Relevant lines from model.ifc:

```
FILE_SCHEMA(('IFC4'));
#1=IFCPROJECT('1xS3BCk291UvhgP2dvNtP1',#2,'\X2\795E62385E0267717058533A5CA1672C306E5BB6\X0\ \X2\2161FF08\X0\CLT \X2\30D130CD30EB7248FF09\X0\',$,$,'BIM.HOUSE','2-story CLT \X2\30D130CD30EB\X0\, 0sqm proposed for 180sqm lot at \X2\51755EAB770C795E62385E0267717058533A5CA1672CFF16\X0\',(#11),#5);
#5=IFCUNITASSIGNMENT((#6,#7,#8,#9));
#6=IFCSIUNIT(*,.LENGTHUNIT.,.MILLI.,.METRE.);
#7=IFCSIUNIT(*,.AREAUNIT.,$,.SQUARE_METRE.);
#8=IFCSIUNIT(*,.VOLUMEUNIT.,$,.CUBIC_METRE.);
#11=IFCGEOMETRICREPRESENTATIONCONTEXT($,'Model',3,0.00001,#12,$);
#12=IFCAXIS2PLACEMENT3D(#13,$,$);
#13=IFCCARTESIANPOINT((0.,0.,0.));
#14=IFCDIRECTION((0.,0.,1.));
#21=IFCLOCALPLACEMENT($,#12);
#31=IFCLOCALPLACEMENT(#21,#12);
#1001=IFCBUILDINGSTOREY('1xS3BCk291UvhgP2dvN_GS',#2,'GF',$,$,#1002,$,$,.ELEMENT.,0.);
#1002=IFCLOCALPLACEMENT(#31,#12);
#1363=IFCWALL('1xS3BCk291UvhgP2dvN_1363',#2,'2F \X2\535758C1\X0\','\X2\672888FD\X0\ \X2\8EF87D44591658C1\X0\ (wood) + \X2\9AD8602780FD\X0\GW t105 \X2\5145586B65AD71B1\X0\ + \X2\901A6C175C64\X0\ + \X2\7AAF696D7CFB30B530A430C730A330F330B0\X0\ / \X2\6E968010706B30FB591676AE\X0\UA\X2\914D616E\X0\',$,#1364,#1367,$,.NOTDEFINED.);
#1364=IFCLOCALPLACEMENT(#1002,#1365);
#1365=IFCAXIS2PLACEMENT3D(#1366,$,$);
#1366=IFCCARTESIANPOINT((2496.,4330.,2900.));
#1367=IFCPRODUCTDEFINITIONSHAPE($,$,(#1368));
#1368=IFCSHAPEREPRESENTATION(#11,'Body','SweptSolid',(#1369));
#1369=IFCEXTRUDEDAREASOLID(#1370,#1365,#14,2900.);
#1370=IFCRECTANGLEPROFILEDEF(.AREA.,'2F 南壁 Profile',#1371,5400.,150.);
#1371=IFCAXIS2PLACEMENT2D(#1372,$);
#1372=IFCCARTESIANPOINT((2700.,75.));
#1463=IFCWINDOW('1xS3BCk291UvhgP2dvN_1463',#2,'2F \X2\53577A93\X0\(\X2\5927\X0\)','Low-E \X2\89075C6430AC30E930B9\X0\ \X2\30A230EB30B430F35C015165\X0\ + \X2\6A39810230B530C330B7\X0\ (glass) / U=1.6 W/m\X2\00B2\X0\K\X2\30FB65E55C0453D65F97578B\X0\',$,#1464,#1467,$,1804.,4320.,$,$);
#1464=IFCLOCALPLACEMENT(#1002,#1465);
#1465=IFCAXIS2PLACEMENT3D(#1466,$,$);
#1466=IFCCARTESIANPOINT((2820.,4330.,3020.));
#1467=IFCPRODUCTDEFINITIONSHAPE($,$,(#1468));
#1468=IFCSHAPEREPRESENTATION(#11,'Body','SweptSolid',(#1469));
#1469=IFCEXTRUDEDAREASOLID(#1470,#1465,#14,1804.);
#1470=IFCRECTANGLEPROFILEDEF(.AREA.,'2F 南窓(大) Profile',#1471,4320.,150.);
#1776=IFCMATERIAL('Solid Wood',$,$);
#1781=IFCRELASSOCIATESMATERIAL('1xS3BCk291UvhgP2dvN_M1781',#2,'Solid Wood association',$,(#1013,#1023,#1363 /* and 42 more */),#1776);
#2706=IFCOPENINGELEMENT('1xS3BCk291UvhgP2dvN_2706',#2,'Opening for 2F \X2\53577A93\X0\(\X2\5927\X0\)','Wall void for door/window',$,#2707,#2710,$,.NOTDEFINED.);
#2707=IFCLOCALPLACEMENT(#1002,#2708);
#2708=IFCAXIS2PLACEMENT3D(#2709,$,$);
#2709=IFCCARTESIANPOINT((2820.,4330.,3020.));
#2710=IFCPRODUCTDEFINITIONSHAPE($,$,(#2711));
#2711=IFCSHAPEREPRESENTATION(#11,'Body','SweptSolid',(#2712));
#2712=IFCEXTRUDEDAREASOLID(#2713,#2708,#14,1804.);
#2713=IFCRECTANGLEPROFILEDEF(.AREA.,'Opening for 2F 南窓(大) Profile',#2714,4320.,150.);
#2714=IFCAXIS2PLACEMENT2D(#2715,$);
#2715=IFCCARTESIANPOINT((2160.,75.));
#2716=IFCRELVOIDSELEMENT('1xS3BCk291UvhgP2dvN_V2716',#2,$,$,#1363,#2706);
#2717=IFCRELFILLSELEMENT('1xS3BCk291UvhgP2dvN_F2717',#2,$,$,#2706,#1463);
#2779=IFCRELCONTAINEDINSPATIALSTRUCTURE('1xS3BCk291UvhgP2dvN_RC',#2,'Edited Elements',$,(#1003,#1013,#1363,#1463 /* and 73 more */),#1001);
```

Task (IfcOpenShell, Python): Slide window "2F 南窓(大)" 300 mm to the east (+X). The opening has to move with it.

```python
import ifcopenshell
import ifcopenshell.api.geometry
import ifcopenshell.util.placement
import ifcopenshell.util.unit

model = ifcopenshell.open("model.ifc")
unit_scale = ifcopenshell.util.unit.calculate_unit_scale(model)

window = model.by_guid("1xS3BCk291UvhgP2dvN_1463")
opening = window.FillsVoids[0].RelatingOpeningElement
wall = opening.VoidsElements[0].RelatingBuildingElement

wall_matrix = ifcopenshell.util.placement.get_local_placement(wall.ObjectPlacement)
shift = wall_matrix[:3, 0] * 0.3 / unit_scale
before = ifcopenshell.util.placement.get_local_placement(window.ObjectPlacement)[:3, 3].copy()

# The window is not placed relative to its opening, so move both.
for product in (opening, window):
    matrix = ifcopenshell.util.placement.get_local_placement(product.ObjectPlacement)
    matrix[:3, 3] += shift
    ifcopenshell.api.geometry.edit_object_placement(model, product=product, matrix=matrix, is_si=False)

after = ifcopenshell.util.placement.get_local_placement(window.ObjectPlacement)[:3, 3]
print("window moved by", (after - before).round(3) + 0.0)

model.write("model_edited.ifc")
```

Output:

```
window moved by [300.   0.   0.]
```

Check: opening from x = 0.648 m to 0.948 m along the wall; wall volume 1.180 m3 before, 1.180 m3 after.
